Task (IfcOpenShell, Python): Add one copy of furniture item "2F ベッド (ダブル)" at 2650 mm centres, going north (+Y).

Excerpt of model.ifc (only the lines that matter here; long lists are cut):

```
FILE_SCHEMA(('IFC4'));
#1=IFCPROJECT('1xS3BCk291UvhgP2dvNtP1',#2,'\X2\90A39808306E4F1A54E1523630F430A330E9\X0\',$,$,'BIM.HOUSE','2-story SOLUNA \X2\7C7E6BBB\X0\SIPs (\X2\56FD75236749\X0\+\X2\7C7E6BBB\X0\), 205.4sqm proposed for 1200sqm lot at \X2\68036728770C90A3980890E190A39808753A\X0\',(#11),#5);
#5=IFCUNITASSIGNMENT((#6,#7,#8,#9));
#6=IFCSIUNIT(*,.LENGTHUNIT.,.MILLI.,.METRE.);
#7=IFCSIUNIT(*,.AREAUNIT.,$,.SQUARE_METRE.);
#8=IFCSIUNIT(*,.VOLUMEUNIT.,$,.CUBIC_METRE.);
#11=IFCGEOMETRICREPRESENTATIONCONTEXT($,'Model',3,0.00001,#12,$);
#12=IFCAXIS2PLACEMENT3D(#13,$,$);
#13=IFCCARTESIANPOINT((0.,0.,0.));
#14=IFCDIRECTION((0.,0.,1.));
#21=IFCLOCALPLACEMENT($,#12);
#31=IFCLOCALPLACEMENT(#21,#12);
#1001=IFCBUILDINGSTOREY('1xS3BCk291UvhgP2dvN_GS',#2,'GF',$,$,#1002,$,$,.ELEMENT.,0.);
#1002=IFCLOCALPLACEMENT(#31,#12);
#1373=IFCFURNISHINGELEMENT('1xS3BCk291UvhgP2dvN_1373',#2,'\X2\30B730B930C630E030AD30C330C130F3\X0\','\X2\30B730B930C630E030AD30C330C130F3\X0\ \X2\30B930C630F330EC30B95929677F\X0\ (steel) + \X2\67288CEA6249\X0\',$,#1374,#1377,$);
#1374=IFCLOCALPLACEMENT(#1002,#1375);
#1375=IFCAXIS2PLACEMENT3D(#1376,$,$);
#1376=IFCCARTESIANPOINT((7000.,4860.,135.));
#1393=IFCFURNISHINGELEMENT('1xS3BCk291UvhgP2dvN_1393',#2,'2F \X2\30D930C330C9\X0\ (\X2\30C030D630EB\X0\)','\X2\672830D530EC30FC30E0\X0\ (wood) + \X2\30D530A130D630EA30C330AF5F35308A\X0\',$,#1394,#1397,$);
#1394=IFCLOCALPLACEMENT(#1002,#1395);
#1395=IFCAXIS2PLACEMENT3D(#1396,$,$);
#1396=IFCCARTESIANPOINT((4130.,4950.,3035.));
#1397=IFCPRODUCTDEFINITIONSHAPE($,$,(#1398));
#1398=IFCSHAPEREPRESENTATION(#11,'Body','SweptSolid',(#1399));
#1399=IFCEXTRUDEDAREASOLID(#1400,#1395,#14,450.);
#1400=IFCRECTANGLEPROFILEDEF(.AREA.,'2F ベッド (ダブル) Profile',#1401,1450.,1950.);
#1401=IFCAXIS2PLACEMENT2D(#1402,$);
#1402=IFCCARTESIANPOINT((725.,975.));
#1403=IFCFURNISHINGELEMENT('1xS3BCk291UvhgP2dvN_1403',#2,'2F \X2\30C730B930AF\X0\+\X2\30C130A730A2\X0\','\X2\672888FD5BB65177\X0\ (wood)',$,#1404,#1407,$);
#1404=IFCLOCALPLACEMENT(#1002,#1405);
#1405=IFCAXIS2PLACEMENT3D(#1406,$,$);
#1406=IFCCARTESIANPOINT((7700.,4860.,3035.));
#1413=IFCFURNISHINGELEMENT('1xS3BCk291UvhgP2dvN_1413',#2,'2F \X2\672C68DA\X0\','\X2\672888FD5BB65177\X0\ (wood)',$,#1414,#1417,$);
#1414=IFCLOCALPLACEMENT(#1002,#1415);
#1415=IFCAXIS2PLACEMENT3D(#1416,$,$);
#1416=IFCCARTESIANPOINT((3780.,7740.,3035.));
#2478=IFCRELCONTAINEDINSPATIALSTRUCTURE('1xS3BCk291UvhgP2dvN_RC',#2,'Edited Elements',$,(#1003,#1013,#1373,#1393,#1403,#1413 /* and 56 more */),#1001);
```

```python
import numpy as np
import ifcopenshell
import ifcopenshell.api.geometry
import ifcopenshell.api.root
import ifcopenshell.util.element
import ifcopenshell.util.placement
import ifcopenshell.util.unit

model = ifcopenshell.open("model.ifc")
unit_scale = ifcopenshell.util.unit.calculate_unit_scale(model)


def reuse_history(source, copy):
    """copy_class also copies each property set's owner history, people and application; keep the originals."""
    for rel in copy.IsDefinedBy:
        if rel.is_a("IfcRelDefinesByProperties") and (history := rel.RelatingPropertyDefinition.OwnerHistory):
            rel.RelatingPropertyDefinition.OwnerHistory = source.OwnerHistory
            ifcopenshell.util.element.remove_deep2(model, history)


source = model.by_guid("1xS3BCk291UvhgP2dvN_1393")
base = ifcopenshell.util.placement.get_local_placement(source.ObjectPlacement)
step = np.array([0.0, 1.0, 0.0]) * 2.65 / unit_scale

for i in range(1, 2):
    copy = ifcopenshell.api.root.copy_class(model, product=source)
    copy.Representation = ifcopenshell.util.element.copy_deep(
        model, source.Representation, exclude=["IfcGeometricRepresentationContext", "IfcRepresentationMap"]
    )
    reuse_history(source, copy)
    matrix = base.copy()
    matrix[:3, 3] += i * step
    print("added at", matrix[:3, 3].round(3) + 0.0)
    ifcopenshell.api.geometry.edit_object_placement(model, product=copy, matrix=matrix, is_si=False)

model.write("model_v2.ifc")
```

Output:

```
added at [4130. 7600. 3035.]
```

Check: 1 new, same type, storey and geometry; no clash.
